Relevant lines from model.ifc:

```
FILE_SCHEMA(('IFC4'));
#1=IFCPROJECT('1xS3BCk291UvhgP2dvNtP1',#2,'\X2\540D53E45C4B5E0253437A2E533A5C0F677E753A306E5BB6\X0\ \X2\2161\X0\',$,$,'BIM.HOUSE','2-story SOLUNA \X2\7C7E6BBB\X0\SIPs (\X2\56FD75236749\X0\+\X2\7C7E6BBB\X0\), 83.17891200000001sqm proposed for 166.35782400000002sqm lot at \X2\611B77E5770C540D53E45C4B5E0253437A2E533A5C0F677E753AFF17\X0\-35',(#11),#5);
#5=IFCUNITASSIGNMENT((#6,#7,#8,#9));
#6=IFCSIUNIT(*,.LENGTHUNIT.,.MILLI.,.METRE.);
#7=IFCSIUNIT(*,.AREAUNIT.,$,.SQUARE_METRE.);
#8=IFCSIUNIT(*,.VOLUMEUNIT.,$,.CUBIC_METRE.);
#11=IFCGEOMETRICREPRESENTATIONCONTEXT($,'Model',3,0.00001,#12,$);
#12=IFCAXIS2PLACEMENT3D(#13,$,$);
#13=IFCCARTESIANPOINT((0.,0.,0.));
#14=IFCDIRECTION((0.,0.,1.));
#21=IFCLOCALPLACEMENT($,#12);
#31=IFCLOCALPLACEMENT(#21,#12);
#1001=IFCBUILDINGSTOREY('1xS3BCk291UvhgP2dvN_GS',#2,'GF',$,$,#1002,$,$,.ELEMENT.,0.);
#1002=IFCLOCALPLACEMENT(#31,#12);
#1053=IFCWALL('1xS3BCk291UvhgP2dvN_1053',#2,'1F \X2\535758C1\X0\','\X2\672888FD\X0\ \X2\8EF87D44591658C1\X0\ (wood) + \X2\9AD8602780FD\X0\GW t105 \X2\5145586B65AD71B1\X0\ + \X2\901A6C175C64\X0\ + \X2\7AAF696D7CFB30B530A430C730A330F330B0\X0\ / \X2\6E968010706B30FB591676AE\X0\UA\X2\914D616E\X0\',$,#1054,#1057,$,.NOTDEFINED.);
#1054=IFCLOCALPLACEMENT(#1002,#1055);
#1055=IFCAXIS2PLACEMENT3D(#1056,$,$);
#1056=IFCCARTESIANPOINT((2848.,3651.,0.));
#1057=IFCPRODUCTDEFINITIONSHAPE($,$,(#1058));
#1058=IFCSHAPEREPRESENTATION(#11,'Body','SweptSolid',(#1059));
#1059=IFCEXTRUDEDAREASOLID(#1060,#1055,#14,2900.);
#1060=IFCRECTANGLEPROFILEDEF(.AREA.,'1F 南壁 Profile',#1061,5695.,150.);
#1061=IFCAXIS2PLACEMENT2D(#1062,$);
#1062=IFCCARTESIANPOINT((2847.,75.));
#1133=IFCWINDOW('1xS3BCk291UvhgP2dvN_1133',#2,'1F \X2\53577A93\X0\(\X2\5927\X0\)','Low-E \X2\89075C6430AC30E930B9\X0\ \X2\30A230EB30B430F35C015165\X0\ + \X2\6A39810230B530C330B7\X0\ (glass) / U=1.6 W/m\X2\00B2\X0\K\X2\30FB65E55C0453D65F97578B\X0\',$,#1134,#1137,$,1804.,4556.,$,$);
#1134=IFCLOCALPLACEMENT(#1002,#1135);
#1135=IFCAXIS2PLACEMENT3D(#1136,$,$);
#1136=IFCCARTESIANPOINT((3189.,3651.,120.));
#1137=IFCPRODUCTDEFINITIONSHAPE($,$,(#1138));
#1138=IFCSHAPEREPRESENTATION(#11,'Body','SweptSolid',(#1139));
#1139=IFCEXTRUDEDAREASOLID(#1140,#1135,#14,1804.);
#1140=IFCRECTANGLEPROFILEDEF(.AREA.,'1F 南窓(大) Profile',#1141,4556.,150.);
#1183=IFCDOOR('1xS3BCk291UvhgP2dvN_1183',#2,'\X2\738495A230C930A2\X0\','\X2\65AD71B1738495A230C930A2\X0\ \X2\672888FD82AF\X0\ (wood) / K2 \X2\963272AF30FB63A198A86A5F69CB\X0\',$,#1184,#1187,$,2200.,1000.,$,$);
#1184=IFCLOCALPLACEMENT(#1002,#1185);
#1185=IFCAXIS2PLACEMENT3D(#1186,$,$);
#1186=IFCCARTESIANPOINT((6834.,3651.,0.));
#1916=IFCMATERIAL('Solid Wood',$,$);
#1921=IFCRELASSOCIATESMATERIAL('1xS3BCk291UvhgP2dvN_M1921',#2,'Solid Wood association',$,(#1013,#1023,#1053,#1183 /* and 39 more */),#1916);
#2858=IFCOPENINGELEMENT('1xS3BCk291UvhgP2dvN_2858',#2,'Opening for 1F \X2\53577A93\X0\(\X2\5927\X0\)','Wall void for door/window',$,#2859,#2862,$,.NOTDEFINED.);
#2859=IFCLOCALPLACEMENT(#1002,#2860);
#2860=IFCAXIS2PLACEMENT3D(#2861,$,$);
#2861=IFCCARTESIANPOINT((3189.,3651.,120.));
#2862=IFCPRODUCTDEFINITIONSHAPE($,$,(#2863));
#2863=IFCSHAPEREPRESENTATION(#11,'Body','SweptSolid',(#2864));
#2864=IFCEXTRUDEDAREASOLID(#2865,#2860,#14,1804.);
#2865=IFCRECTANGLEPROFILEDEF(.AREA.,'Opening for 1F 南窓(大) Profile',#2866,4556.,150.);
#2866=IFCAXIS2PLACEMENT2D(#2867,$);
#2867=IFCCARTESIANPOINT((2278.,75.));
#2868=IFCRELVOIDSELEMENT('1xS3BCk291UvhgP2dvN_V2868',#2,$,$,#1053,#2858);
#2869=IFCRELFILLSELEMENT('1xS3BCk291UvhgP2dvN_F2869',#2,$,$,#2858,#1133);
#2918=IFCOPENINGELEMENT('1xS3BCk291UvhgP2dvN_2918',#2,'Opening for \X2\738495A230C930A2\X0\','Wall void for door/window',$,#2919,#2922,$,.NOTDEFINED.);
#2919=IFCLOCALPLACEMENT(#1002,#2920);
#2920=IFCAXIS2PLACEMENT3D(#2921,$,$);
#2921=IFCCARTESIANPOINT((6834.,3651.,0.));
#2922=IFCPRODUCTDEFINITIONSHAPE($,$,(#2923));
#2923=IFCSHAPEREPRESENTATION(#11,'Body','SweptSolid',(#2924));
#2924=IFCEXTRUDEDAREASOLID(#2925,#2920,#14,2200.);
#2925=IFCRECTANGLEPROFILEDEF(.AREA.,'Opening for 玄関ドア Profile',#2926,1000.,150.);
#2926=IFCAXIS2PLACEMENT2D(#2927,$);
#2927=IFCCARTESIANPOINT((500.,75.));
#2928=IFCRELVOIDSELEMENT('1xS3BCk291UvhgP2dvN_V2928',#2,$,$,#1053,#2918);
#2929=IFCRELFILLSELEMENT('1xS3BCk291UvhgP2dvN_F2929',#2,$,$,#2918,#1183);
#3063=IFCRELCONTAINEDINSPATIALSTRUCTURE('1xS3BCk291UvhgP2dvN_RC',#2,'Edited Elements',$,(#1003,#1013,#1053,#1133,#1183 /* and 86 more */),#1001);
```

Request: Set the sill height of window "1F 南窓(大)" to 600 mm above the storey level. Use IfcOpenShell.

```python
import numpy as np
import ifcopenshell
import ifcopenshell.api.geometry
import ifcopenshell.geom
import ifcopenshell.util.element
import ifcopenshell.util.placement
import ifcopenshell.util.shape
import ifcopenshell.util.unit

model = ifcopenshell.open("model.ifc")
unit_scale = ifcopenshell.util.unit.calculate_unit_scale(model)

window = model.by_guid("1xS3BCk291UvhgP2dvN_1133")
opening = window.FillsVoids[0].RelatingOpeningElement
storey = ifcopenshell.util.element.get_container(window, ifc_class="IfcBuildingStorey")
level = ifcopenshell.util.placement.get_local_placement(storey.ObjectPlacement)[2, 3]

# The opening's origin need not be at the sill, so measure its lowest point.
shape = ifcopenshell.geom.create_shape(ifcopenshell.geom.settings(), opening)
bottom = ifcopenshell.util.shape.get_shape_bottom_elevation(shape, shape.geometry) / unit_scale
dz = level + 0.6 / unit_scale - bottom

shift = np.array([0.0, 0.0, dz])
# The window is not placed relative to its opening, so move both.
for product in (opening, window):
    matrix = ifcopenshell.util.placement.get_local_placement(product.ObjectPlacement)
    matrix[:3, 3] += shift
    ifcopenshell.api.geometry.edit_object_placement(model, product=product, matrix=matrix, is_si=False)

print(f"moved by {dz * unit_scale:+.3f} m")

model.write("model_updated.ifc")
```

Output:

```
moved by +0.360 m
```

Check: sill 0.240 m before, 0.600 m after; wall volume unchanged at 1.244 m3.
